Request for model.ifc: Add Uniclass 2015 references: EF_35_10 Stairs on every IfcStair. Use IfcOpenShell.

First a look at what the model holds.

```python
import ifcopenshell

model = ifcopenshell.open("model.ifc")
print(model.schema)
print("classifications:", [c.Name for c in model.by_type("IfcClassification")])
for ifc_class in ("IfcDoor", "IfcRoof", "IfcStair", "IfcWall", "IfcWindow"):
    print(ifc_class, len(model.by_type(ifc_class)))
```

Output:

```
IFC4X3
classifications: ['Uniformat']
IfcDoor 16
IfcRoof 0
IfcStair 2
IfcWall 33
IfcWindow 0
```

```python
import ifcopenshell
import ifcopenshell.api.classification

model = ifcopenshell.open("model.ifc")

system = ifcopenshell.api.classification.add_classification(model, classification="Uniclass 2015")

codes = {
    "IfcStair": ("EF_35_10", "Stairs"),
}
for ifc_class, (code, name) in codes.items():
    products = model.by_type(ifc_class)
    ifcopenshell.api.classification.add_reference(
        model, products=products, classification=system, identification=code, name=name
    )
    print(code, len(products))

model.write("model_updated.ifc")
```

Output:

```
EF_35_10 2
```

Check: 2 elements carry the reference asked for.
